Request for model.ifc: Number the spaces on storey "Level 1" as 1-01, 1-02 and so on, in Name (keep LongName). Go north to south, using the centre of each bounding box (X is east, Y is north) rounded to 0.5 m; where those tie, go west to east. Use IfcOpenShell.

First a look at what the model holds.

```python
import ifcopenshell
import ifcopenshell.util.element
import ifcopenshell.util.placement

model = ifcopenshell.open("model.ifc")
print(model.schema)
storey = next(s for s in model.by_type("IfcBuildingStorey") if s.Name == "Level 1")
spaces = [e for e in ifcopenshell.util.element.get_decomposition(storey) if e.is_a("IfcSpace")]
for e in sorted(spaces, key=lambda e: e.id()):
    origin = ifcopenshell.util.placement.get_local_placement(e.ObjectPlacement)[:3, 3]
    print(e.id(), e.Name, e.LongName, origin.round(2) + 0.0, sep=" | ")
```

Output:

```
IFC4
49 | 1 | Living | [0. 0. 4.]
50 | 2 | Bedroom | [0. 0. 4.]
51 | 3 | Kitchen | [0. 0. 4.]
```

```python
import ifcopenshell
import ifcopenshell.geom
import ifcopenshell.util.element
import ifcopenshell.util.shape

model = ifcopenshell.open("model.ifc")
settings = ifcopenshell.geom.settings()
settings.set("use-world-coords", True)


def centre(element):
    shape = ifcopenshell.geom.create_shape(settings, element)
    return ifcopenshell.util.shape.get_bbox_centroid(shape.geometry)


storey = next(s for s in model.by_type("IfcBuildingStorey") if s.Name == "Level 1")
spaces = [e for e in ifcopenshell.util.element.get_decomposition(storey) if e.is_a("IfcSpace")]

# Insertion points can sit at a corner or the storey origin, so sort by the geometry (in metres).
centres = {e: centre(e) for e in spaces}
spaces.sort(key=lambda e: (-round(centres[e][1] / 0.5), centres[e][0]))

for i, e in enumerate(spaces, start=1):
    number = f"1-{i:02d}"
    e.Name = number
    print(e.id(), number)

model.write("model_rev.ifc")
```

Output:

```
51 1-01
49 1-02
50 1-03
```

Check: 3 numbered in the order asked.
